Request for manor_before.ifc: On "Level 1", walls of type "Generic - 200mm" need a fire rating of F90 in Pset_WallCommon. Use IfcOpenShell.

First a look at what the model holds.

```python
import ifcopenshell
import ifcopenshell.util.element

model = ifcopenshell.open("manor_before.ifc")
print(model.schema)
storey = next(s for s in model.by_type("IfcBuildingStorey") if s.Name == "Level 1")
walls = [e for e in ifcopenshell.util.element.get_decomposition(storey) if e.is_a("IfcWall")]
seen = {}
for e in walls:
    element_type = ifcopenshell.util.element.get_type(e)
    key = (element_type.Name if element_type != e and element_type else None, ifcopenshell.util.element.get_pset(e, "Pset_WallCommon", "FireRating"))
    seen[key] = seen.get(key, 0) + 1
for (name, value), count in sorted(seen.items(), key=str):
    print(count, "x", name, "|", value)
```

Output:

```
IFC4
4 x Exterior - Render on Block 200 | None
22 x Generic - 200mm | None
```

```python
import ifcopenshell
import ifcopenshell.api.pset
import ifcopenshell.util.element

model = ifcopenshell.open("manor_before.ifc")

storey = next(s for s in model.by_type("IfcBuildingStorey") if s.Name == "Level 1")
walls = [e for e in ifcopenshell.util.element.get_decomposition(storey) if e.is_a("IfcWall")]

count = 0
for e in walls:
    element_type = ifcopenshell.util.element.get_type(e)
    if element_type in (None, e) or element_type.Name != "Generic - 200mm":
        continue
    # add_pset returns the element's existing set when there is one.
    pset = ifcopenshell.api.pset.add_pset(model, product=e, name="Pset_WallCommon")
    ifcopenshell.api.pset.edit_pset(model, pset=pset, properties={"FireRating": "F90"})
    count += 1

print(count, "walls updated")

model.write("manor_before_rev.ifc")
```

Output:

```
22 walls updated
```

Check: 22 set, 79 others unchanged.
